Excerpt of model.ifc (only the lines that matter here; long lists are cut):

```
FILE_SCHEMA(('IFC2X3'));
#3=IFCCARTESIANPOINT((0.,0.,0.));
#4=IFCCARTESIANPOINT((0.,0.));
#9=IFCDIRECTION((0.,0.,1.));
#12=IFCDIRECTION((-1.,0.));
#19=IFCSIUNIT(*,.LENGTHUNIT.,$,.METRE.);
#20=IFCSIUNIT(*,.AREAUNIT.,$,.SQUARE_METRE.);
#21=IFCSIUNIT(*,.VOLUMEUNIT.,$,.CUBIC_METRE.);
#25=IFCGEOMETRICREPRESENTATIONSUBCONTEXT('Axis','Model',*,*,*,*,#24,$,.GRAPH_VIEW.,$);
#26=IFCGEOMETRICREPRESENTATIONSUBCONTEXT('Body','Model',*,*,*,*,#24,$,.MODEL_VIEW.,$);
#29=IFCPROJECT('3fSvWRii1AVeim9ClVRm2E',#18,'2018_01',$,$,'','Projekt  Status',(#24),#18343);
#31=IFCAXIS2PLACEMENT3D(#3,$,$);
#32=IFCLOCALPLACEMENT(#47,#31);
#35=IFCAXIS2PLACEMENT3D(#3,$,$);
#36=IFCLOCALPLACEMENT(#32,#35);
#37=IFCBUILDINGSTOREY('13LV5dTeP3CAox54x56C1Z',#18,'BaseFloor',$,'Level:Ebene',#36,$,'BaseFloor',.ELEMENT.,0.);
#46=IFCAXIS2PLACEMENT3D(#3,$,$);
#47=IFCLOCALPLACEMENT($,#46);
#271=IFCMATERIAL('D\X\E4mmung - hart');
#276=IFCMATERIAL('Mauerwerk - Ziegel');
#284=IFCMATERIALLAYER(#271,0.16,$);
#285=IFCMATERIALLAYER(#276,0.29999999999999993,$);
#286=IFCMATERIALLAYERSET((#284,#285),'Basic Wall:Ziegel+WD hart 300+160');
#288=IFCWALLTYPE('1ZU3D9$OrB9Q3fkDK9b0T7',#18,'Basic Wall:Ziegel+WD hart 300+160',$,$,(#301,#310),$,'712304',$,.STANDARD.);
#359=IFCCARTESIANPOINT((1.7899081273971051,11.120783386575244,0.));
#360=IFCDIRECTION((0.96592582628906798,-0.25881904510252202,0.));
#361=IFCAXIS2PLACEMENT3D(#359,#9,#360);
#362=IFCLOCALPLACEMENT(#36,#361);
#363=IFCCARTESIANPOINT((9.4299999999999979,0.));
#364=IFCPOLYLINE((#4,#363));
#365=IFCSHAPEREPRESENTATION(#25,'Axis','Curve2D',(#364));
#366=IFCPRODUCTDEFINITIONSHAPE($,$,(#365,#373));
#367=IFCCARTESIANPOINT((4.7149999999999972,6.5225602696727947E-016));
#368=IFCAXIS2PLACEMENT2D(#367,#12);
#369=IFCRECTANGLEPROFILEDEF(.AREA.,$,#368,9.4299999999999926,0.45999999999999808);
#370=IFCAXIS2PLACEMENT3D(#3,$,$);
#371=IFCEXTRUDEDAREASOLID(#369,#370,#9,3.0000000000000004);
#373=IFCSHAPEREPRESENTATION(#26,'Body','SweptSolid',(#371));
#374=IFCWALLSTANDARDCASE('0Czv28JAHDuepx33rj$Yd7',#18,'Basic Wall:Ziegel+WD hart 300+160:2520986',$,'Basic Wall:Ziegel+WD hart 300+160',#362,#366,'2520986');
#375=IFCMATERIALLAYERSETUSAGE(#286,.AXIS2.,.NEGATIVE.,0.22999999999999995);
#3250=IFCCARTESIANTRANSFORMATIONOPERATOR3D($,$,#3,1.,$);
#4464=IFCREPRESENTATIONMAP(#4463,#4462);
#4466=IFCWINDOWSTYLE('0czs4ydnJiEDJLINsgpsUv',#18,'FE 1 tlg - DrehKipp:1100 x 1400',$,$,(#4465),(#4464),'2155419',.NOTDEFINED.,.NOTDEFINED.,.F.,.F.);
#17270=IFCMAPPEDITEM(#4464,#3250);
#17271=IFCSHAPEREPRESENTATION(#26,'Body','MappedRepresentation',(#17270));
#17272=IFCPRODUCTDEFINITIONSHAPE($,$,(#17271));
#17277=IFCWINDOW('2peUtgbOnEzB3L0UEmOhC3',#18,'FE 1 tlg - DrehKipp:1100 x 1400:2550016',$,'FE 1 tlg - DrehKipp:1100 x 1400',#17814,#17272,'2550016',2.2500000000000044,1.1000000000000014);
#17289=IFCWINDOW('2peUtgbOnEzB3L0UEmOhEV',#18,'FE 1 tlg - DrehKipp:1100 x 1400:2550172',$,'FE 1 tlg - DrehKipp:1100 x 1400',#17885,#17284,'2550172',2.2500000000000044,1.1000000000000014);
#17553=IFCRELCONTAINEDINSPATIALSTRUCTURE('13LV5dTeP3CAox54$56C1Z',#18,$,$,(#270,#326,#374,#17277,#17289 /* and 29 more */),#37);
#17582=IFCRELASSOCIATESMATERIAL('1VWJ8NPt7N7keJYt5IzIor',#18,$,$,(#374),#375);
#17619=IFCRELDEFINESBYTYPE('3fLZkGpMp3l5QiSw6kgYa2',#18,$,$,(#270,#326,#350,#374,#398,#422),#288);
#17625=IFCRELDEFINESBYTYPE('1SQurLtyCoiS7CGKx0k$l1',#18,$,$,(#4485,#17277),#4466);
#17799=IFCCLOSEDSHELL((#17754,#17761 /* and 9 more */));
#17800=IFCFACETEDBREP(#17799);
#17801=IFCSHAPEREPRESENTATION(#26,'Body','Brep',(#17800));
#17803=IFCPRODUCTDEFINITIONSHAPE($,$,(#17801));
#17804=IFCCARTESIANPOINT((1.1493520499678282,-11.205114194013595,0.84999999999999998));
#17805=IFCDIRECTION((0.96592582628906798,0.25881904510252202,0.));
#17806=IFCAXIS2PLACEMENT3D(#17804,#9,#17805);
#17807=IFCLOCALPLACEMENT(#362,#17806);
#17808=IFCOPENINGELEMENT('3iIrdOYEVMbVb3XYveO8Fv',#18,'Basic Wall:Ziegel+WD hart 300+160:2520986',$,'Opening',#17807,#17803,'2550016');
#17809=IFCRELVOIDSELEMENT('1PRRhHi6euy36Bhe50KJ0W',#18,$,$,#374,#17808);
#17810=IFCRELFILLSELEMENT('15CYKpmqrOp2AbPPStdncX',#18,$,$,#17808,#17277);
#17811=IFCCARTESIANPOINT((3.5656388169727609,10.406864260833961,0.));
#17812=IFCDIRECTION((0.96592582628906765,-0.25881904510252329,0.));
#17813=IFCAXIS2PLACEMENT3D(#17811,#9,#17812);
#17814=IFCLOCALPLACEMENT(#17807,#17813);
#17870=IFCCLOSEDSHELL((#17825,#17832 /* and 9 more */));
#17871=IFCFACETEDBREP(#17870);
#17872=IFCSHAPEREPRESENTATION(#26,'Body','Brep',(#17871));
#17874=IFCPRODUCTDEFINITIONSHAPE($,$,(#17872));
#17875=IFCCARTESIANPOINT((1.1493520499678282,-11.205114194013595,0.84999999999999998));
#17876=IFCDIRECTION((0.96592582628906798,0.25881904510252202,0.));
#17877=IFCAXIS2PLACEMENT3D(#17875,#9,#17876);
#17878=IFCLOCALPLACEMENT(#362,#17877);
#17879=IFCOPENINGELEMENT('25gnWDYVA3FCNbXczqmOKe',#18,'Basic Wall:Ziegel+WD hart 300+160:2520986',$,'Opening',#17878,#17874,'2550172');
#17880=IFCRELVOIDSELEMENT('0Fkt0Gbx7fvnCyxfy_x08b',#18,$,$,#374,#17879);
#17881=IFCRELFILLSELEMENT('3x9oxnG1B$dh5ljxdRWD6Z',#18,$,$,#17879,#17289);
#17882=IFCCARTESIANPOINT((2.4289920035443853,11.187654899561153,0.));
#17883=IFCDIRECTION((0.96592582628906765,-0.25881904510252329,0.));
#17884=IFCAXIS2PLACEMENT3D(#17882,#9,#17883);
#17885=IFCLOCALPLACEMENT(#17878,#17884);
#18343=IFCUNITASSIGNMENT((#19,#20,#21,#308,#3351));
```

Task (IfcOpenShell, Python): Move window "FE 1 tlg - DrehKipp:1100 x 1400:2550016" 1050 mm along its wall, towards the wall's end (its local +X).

```python
import ifcopenshell
import ifcopenshell.api.geometry
import ifcopenshell.util.placement

model = ifcopenshell.open("model.ifc")

window = model.by_guid("2peUtgbOnEzB3L0UEmOhC3")
opening = window.FillsVoids[0].RelatingOpeningElement
wall = opening.VoidsElements[0].RelatingBuildingElement

wall_matrix = ifcopenshell.util.placement.get_local_placement(wall.ObjectPlacement)
shift = wall_matrix[:3, 0] * 1.05
before = ifcopenshell.util.placement.get_local_placement(window.ObjectPlacement)[:3, 3].copy()

# The window is placed relative to its opening, so it follows when the opening moves.
matrix = ifcopenshell.util.placement.get_local_placement(opening.ObjectPlacement)
matrix[:3, 3] += shift
ifcopenshell.api.geometry.edit_object_placement(
    model, product=opening, matrix=matrix, is_si=False, should_transform_children=True
)

after = ifcopenshell.util.placement.get_local_placement(window.ObjectPlacement)[:3, 3]
print("window moved by", (after - before).round(3) + 0.0)

model.write("model_updated.ifc")
```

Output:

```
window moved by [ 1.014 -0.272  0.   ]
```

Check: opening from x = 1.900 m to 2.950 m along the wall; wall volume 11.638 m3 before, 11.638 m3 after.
